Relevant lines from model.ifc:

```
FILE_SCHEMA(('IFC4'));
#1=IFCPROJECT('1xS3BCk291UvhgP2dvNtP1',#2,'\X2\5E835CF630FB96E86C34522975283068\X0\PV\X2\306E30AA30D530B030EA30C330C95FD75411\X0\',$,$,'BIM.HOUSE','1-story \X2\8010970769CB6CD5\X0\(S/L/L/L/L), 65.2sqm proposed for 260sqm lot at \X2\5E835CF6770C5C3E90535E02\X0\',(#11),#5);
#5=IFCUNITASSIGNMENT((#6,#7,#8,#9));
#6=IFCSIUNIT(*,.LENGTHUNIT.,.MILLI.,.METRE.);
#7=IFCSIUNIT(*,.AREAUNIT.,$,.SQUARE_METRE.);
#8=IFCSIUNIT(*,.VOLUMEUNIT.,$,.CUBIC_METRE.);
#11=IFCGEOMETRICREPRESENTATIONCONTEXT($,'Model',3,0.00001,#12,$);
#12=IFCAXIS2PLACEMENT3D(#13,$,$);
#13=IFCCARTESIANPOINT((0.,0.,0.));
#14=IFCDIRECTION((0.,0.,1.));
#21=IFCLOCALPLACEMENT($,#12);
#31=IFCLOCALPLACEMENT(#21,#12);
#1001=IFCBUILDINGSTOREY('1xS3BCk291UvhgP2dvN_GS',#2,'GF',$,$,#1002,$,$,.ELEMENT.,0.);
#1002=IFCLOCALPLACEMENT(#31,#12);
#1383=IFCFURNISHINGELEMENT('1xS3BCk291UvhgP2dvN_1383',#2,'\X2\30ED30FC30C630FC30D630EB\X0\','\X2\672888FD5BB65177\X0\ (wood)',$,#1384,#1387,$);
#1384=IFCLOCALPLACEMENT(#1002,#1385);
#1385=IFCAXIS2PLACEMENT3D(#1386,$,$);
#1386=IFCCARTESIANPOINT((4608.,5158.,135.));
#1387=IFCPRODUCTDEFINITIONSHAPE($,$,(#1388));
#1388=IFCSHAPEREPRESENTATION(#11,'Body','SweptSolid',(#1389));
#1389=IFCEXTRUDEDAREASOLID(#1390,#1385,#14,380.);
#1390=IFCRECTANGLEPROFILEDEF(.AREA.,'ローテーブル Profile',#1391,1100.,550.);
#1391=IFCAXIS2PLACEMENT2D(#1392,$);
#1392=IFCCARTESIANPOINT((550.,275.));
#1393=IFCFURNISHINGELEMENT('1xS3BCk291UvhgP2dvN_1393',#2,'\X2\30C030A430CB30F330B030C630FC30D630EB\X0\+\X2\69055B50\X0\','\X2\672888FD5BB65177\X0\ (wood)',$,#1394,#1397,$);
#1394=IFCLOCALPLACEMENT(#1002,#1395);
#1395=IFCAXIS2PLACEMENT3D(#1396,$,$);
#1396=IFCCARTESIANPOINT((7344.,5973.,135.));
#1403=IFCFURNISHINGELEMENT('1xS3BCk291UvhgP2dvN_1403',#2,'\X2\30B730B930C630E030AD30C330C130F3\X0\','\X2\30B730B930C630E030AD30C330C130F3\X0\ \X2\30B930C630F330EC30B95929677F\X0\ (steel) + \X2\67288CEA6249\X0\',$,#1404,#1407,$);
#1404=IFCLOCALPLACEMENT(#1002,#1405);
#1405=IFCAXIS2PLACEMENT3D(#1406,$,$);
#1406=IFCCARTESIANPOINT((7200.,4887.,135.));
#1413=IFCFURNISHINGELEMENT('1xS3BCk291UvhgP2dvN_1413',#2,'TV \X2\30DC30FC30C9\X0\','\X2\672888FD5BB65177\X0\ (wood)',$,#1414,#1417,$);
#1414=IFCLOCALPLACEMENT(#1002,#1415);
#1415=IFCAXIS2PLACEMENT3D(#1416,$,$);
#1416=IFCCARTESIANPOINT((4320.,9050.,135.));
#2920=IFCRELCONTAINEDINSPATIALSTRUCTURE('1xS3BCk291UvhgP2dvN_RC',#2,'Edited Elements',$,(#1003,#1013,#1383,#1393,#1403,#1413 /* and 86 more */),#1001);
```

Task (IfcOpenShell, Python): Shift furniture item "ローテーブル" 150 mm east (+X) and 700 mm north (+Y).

```python
import ifcopenshell
import ifcopenshell.api.geometry
import ifcopenshell.util.placement

model = ifcopenshell.open("model.ifc")

item = model.by_id(1383)
matrix = ifcopenshell.util.placement.get_local_placement(item.ObjectPlacement)
matrix[0, 3] += 150.0
matrix[1, 3] += 700.0
ifcopenshell.api.geometry.edit_object_placement(model, product=item, matrix=matrix, is_si=False)

print(ifcopenshell.util.placement.get_local_placement(item.ObjectPlacement).round(3) + 0.0)

model.write("model_edited.ifc")
```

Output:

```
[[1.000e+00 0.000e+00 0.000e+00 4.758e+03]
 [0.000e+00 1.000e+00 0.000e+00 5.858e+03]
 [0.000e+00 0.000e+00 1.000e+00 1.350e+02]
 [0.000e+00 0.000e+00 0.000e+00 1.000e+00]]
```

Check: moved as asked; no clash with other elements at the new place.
